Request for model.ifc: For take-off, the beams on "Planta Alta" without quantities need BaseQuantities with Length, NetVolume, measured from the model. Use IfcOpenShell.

First a look at what the model holds.

```python
import ifcopenshell
import ifcopenshell.util.element
import ifcopenshell.util.unit

model = ifcopenshell.open("model.ifc")
print(model.schema)
for unit_type in ("LENGTHUNIT", "AREAUNIT", "VOLUMEUNIT"):
    print(unit_type, ifcopenshell.util.unit.calculate_unit_scale(model, unit_type))
storey = next(s for s in model.by_type("IfcBuildingStorey") if s.Name == "Planta Alta")
beams = [e for e in ifcopenshell.util.element.get_decomposition(storey) if e.is_a("IfcBeam")]
for e in sorted(beams, key=lambda e: e.id()):
    print(e.id(), e.is_a(), e.Name, list(ifcopenshell.util.element.get_psets(e, qtos_only=True)), sep=" | ")
```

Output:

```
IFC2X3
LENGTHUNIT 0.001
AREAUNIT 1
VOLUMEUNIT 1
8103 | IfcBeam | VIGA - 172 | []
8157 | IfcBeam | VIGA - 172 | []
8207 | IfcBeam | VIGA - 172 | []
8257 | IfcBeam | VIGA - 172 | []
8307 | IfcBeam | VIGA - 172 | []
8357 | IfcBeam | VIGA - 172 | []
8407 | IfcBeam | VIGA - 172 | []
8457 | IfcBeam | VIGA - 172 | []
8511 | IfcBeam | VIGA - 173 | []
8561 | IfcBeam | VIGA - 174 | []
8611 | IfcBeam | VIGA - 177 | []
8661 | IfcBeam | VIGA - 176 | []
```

```python
import ifcopenshell
import ifcopenshell.api.pset
import ifcopenshell.geom
import ifcopenshell.util.element
import ifcopenshell.util.shape
import ifcopenshell.util.unit

model = ifcopenshell.open("model.ifc")
unit_scale = ifcopenshell.util.unit.calculate_unit_scale(model)
volume_scale = ifcopenshell.util.unit.calculate_unit_scale(model, "VOLUMEUNIT")
settings = ifcopenshell.geom.settings()

storey = next(s for s in model.by_type("IfcBuildingStorey") if s.Name == "Planta Alta")
beams = [e for e in ifcopenshell.util.element.get_decomposition(storey) if e.is_a("IfcBeam")]

for e in sorted(beams, key=lambda e: e.id()):
    if ifcopenshell.util.element.get_psets(e, qtos_only=True, should_inherit=False):
        continue
    # Geometry comes back in metres, in the element's own axes.
    shape = ifcopenshell.geom.create_shape(settings, e)
    values = {
        "Length": ifcopenshell.util.shape.get_max_xyz(shape.geometry) / unit_scale,
        "NetVolume": ifcopenshell.util.shape.get_volume(shape.geometry) / volume_scale,
    }
    qto = ifcopenshell.api.pset.add_qto(model, product=e, name="BaseQuantities")
    ifcopenshell.api.pset.edit_qto(model, qto=qto, properties=values)
    print(e.id(), {k: round(v, 3) for k, v in values.items()})

model.write("model_rev.ifc")
```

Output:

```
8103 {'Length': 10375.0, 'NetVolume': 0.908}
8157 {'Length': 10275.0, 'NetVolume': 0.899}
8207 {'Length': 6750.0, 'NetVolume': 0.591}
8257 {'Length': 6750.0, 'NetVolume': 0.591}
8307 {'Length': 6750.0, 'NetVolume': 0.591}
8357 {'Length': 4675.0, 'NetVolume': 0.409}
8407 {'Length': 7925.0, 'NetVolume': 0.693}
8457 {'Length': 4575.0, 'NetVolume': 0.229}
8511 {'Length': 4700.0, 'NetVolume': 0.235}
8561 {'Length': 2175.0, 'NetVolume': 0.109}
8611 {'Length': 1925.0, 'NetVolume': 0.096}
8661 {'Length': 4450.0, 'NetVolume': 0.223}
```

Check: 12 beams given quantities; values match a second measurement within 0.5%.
